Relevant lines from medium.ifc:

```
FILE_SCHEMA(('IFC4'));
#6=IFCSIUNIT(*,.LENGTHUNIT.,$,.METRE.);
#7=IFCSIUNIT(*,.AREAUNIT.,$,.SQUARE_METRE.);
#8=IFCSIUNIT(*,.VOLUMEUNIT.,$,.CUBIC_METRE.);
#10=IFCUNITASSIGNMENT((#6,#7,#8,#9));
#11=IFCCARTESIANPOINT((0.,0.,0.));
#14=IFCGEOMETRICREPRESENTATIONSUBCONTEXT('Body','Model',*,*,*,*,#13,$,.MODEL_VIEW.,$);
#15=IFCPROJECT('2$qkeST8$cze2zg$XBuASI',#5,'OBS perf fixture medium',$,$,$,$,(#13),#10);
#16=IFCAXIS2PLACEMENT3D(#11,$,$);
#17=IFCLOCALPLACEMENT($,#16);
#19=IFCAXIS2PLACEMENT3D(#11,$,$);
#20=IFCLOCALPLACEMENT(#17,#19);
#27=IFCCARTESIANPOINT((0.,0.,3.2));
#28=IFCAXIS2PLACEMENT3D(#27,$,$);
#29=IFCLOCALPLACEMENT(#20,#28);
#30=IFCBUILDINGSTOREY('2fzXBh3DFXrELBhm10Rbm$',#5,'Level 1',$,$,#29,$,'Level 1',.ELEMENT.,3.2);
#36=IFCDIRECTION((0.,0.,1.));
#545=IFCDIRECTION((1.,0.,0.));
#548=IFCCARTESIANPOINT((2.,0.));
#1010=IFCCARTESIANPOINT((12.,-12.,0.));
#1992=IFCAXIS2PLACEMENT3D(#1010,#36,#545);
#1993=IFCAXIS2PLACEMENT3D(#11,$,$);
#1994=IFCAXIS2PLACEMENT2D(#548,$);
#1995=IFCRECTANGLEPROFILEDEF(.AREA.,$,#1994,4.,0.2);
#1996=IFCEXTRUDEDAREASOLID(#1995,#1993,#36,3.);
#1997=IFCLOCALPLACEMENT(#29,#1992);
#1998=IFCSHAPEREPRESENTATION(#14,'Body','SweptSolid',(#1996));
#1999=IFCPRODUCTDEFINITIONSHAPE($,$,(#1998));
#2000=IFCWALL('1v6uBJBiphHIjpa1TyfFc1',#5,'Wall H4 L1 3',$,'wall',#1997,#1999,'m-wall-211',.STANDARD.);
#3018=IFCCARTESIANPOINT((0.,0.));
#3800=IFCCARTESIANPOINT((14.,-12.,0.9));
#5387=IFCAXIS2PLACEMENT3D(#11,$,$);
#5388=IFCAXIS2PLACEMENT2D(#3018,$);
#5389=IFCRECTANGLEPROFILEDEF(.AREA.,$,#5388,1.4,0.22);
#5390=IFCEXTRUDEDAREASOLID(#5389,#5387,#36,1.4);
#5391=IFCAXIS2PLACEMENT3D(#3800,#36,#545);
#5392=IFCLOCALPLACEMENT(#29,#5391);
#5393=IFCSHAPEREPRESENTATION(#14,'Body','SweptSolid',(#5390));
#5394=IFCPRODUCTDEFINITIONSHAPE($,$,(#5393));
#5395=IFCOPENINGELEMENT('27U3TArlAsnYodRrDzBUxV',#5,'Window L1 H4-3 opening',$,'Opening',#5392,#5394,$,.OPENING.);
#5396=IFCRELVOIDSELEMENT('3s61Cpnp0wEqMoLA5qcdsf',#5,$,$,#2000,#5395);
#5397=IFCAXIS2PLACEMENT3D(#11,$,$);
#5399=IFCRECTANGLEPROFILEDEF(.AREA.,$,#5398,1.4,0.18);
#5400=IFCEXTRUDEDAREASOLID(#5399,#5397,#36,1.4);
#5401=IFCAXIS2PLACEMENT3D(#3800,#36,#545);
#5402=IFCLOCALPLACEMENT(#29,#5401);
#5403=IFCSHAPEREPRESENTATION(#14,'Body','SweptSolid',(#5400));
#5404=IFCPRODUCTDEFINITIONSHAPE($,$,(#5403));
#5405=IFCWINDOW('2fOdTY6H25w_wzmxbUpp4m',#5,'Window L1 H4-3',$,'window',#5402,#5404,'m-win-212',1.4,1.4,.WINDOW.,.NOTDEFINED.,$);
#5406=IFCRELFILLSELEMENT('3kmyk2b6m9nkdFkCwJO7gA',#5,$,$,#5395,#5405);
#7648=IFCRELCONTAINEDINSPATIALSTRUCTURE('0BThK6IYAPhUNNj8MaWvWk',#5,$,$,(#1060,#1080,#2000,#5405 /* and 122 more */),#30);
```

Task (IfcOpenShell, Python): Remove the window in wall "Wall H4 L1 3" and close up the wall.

```python
import ifcopenshell
import ifcopenshell.api.feature
import ifcopenshell.api.root
import ifcopenshell.geom
import ifcopenshell.util.shape

model = ifcopenshell.open("medium.ifc")
settings = ifcopenshell.geom.settings()


def volume(element):
    """Net volume in cubic metres, openings subtracted."""
    shape = ifcopenshell.geom.create_shape(settings, element)
    return ifcopenshell.util.shape.get_volume(shape.geometry)


window = model.by_id(5405)
opening = window.FillsVoids[0].RelatingOpeningElement
wall = opening.VoidsElements[0].RelatingBuildingElement
before = volume(wall)

ifcopenshell.api.root.remove_product(model, product=window)
ifcopenshell.api.feature.remove_feature(model, feature=opening)

after = volume(wall)

print(f"wall volume {before:.3f} -> {after:.3f} m3")

model.write("medium-out.ifc")
```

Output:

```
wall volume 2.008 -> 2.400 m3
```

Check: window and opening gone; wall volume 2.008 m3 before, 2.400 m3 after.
